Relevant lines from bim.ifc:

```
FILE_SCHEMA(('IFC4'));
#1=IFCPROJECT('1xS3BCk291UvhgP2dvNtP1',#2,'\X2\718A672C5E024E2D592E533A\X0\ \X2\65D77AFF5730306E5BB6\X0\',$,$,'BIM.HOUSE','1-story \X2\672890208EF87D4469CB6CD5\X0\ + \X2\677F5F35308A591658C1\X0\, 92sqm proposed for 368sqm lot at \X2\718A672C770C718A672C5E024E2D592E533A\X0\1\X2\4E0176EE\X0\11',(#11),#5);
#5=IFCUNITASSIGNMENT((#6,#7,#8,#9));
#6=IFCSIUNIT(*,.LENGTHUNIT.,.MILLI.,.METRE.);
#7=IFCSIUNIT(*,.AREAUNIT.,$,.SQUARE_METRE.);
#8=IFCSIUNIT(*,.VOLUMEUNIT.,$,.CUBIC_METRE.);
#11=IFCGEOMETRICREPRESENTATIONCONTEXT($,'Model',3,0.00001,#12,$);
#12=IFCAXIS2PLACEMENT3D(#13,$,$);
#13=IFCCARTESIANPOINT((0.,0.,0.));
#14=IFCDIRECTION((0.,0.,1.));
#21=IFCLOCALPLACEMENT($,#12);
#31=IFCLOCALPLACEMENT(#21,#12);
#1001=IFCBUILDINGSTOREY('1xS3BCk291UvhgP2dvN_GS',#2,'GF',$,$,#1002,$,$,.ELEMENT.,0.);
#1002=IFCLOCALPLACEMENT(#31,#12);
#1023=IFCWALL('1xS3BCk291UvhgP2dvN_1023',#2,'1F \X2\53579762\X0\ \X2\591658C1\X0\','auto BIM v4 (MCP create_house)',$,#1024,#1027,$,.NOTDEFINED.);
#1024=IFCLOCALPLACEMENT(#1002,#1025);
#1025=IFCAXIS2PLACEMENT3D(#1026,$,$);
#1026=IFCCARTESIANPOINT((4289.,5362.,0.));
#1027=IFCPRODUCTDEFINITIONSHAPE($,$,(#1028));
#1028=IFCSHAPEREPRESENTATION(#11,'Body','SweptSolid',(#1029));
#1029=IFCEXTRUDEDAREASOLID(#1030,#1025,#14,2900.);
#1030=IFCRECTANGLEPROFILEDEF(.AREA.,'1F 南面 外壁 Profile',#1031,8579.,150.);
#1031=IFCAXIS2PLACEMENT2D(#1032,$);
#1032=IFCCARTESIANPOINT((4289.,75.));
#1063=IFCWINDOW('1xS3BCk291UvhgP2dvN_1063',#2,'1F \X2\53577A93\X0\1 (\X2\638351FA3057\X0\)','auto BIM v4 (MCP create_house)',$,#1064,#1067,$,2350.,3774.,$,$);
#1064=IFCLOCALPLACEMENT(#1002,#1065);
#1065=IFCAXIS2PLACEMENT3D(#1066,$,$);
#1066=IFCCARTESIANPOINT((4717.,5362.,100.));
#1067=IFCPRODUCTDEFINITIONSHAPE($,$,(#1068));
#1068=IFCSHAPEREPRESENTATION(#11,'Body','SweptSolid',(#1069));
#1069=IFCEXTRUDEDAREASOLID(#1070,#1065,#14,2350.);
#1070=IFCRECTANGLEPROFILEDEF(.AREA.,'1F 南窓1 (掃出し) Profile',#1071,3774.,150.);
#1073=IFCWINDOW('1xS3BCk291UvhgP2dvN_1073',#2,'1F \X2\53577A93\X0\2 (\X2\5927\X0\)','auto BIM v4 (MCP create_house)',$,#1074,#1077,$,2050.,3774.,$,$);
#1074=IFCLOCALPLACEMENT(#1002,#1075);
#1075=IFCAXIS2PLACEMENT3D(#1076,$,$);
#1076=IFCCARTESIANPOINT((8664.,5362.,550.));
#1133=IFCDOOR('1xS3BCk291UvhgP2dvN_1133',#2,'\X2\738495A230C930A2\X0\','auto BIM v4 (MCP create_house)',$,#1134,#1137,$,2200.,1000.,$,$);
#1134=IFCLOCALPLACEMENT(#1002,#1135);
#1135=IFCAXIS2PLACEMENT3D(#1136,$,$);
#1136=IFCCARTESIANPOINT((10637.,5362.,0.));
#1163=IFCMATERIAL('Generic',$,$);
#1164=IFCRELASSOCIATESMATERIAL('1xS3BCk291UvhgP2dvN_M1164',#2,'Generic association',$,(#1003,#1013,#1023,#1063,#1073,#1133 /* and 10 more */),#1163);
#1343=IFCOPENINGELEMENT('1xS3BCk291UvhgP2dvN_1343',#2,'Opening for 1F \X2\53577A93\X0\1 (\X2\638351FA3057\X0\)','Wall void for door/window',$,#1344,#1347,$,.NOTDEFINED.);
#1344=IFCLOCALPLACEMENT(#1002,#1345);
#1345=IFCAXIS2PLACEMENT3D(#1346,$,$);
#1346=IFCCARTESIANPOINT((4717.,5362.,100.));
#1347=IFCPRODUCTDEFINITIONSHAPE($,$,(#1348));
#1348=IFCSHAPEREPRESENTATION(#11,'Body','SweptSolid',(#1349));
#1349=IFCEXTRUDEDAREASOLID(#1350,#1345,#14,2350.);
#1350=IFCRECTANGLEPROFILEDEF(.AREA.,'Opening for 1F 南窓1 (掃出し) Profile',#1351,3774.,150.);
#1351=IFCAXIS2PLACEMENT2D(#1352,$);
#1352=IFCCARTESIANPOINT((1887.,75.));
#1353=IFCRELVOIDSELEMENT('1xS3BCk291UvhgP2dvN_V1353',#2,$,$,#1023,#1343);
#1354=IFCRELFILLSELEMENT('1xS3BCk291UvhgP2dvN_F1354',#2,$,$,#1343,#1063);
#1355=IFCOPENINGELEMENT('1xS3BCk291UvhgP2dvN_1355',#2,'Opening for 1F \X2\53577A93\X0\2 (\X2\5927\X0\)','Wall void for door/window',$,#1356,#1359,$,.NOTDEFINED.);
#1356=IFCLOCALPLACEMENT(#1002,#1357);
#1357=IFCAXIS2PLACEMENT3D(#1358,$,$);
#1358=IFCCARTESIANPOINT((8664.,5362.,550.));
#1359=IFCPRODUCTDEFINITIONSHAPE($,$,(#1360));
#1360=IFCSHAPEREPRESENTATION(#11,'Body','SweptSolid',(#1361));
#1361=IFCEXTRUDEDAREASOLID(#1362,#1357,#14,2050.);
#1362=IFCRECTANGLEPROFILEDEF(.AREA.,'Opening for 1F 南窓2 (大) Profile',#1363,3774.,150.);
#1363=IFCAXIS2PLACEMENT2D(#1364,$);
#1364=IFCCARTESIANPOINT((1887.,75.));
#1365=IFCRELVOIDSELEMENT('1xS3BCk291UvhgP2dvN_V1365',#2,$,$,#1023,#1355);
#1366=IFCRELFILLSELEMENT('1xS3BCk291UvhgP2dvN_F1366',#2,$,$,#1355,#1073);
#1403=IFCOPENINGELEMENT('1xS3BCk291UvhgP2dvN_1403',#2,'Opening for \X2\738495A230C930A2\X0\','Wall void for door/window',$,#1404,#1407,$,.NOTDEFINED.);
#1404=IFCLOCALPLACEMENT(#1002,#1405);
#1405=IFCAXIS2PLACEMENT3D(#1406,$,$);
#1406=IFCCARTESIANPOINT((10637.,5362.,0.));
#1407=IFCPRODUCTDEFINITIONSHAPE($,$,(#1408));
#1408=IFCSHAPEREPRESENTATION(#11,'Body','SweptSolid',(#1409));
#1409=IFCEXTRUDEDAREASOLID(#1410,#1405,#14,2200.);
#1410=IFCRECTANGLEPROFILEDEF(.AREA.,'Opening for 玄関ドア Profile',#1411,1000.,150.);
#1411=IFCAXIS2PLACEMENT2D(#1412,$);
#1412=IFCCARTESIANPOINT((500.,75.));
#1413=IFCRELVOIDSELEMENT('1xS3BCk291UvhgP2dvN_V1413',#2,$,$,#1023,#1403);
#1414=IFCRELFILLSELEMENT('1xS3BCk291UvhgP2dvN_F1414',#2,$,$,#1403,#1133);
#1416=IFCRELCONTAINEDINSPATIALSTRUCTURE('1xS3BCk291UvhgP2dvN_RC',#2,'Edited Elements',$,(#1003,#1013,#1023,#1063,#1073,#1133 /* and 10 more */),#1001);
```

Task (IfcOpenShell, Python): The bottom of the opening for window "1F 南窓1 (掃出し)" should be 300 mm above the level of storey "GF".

```python
import numpy as np
import ifcopenshell
import ifcopenshell.api.geometry
import ifcopenshell.geom
import ifcopenshell.util.element
import ifcopenshell.util.placement
import ifcopenshell.util.shape
import ifcopenshell.util.unit

model = ifcopenshell.open("bim.ifc")
unit_scale = ifcopenshell.util.unit.calculate_unit_scale(model)

window = model.by_guid("1xS3BCk291UvhgP2dvN_1063")
opening = window.FillsVoids[0].RelatingOpeningElement
storey = ifcopenshell.util.element.get_container(window, ifc_class="IfcBuildingStorey")
level = ifcopenshell.util.placement.get_local_placement(storey.ObjectPlacement)[2, 3]

# The opening's origin need not be at the sill, so measure its lowest point.
shape = ifcopenshell.geom.create_shape(ifcopenshell.geom.settings(), opening)
bottom = ifcopenshell.util.shape.get_shape_bottom_elevation(shape, shape.geometry) / unit_scale
dz = level + 0.3 / unit_scale - bottom

shift = np.array([0.0, 0.0, dz])
# The window is not placed relative to its opening, so move both.
for product in (opening, window):
    matrix = ifcopenshell.util.placement.get_local_placement(product.ObjectPlacement)
    matrix[:3, 3] += shift
    ifcopenshell.api.geometry.edit_object_placement(model, product=product, matrix=matrix, is_si=False)

print(f"moved by {dz * unit_scale:+.3f} m")

model.write("bim-out.ifc")
```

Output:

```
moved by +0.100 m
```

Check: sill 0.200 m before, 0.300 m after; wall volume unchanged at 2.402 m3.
